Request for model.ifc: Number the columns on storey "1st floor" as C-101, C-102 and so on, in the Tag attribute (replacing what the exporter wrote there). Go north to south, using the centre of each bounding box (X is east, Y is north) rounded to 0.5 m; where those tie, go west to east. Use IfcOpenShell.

First a look at what the model holds.

```python
import ifcopenshell
import ifcopenshell.util.element
import ifcopenshell.util.placement

model = ifcopenshell.open("model.ifc")
print(model.schema)
storey = next(s for s in model.by_type("IfcBuildingStorey") if s.Name == "1st floor")
columns = [e for e in ifcopenshell.util.element.get_decomposition(storey) if e.is_a("IfcColumn")]
for e in sorted(columns, key=lambda e: e.id()):
    origin = ifcopenshell.util.placement.get_local_placement(e.ObjectPlacement)[:3, 3]
    print(e.id(), e.Tag, e.Name, origin.round(2) + 0.0, sep=" | ")
```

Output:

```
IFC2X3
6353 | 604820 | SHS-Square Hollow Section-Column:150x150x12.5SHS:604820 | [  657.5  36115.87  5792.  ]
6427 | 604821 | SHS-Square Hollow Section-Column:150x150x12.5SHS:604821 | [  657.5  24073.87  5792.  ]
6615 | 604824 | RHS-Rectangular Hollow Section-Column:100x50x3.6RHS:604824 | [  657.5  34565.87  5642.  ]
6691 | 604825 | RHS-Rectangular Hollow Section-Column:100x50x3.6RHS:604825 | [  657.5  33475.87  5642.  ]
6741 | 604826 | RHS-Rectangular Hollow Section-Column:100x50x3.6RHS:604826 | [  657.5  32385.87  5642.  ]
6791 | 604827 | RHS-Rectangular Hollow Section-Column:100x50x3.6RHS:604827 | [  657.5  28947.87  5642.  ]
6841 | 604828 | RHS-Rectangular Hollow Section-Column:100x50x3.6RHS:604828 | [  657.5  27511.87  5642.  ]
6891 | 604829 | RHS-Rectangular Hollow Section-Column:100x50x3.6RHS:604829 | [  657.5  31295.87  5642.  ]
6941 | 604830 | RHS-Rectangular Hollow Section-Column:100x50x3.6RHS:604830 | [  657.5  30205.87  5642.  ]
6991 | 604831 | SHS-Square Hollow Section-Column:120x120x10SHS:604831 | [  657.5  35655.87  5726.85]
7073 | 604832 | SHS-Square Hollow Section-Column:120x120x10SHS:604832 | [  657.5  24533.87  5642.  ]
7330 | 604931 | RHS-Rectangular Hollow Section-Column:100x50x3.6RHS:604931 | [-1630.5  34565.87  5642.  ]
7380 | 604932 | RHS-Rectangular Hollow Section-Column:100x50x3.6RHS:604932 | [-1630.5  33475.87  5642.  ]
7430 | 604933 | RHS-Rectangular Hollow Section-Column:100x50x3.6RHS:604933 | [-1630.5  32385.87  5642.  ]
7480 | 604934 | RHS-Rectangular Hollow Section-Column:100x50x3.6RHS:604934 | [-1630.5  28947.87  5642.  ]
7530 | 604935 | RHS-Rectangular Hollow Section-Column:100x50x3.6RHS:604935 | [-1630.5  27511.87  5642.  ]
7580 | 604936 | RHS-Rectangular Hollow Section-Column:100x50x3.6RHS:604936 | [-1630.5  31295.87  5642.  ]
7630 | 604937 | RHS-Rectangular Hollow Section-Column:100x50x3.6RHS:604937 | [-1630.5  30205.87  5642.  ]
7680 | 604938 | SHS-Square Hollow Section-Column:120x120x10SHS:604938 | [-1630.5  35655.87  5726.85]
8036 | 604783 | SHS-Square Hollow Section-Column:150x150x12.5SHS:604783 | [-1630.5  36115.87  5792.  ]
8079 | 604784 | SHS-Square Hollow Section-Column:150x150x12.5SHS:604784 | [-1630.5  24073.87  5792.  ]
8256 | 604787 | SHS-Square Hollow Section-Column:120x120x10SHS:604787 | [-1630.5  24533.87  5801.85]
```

```python
import ifcopenshell
import ifcopenshell.geom
import ifcopenshell.util.element
import ifcopenshell.util.shape

model = ifcopenshell.open("model.ifc")
settings = ifcopenshell.geom.settings()
settings.set("use-world-coords", True)


def centre(element):
    shape = ifcopenshell.geom.create_shape(settings, element)
    return ifcopenshell.util.shape.get_bbox_centroid(shape.geometry)


storey = next(s for s in model.by_type("IfcBuildingStorey") if s.Name == "1st floor")
columns = [e for e in ifcopenshell.util.element.get_decomposition(storey) if e.is_a("IfcColumn")]

# Insertion points can sit at a corner or the storey origin, so sort by the geometry (in metres).
centres = {e: centre(e) for e in columns}
columns.sort(key=lambda e: (-round(centres[e][1] / 0.5), centres[e][0]))

for i, e in enumerate(columns, start=1):
    number = f"C-1{i:02d}"
    e.Tag = number
    print(e.id(), number)

model.write("model_edited.ifc")
```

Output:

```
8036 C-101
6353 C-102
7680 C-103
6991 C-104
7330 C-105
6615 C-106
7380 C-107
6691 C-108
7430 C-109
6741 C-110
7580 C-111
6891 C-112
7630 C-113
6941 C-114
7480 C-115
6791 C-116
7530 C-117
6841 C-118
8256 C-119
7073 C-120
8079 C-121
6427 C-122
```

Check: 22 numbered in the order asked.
